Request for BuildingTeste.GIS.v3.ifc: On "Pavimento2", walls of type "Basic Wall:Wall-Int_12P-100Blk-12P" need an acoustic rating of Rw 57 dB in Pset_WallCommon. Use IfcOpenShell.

First a look at what the model holds.

```python
import ifcopenshell
import ifcopenshell.util.element

model = ifcopenshell.open("BuildingTeste.GIS.v3.ifc")
print(model.schema)
storey = next(s for s in model.by_type("IfcBuildingStorey") if s.Name == "Pavimento2")
walls = [e for e in ifcopenshell.util.element.get_decomposition(storey) if e.is_a("IfcWall")]
seen = {}
for e in walls:
    element_type = ifcopenshell.util.element.get_type(e)
    key = (element_type.Name if element_type != e and element_type else None, ifcopenshell.util.element.get_pset(e, "Pset_WallCommon", "AcousticRating"))
    seen[key] = seen.get(key, 0) + 1
for (name, value), count in sorted(seen.items(), key=str):
    print(count, "x", name, "|", value)
```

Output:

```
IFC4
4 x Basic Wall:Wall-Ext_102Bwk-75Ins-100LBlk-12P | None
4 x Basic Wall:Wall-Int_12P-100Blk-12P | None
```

```python
import ifcopenshell
import ifcopenshell.api.pset
import ifcopenshell.util.element

model = ifcopenshell.open("BuildingTeste.GIS.v3.ifc")

storey = next(s for s in model.by_type("IfcBuildingStorey") if s.Name == "Pavimento2")
walls = [e for e in ifcopenshell.util.element.get_decomposition(storey) if e.is_a("IfcWall")]

count = 0
for e in walls:
    element_type = ifcopenshell.util.element.get_type(e)
    if element_type in (None, e) or element_type.Name != "Basic Wall:Wall-Int_12P-100Blk-12P":
        continue
    # add_pset returns the element's existing set when there is one.
    pset = ifcopenshell.api.pset.add_pset(model, product=e, name="Pset_WallCommon")
    ifcopenshell.api.pset.edit_pset(model, pset=pset, properties={"AcousticRating": "Rw 57 dB"})
    count += 1

print(count, "walls updated")

model.write("BuildingTeste.GIS.v3-out.ifc")
```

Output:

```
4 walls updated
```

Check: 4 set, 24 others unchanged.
